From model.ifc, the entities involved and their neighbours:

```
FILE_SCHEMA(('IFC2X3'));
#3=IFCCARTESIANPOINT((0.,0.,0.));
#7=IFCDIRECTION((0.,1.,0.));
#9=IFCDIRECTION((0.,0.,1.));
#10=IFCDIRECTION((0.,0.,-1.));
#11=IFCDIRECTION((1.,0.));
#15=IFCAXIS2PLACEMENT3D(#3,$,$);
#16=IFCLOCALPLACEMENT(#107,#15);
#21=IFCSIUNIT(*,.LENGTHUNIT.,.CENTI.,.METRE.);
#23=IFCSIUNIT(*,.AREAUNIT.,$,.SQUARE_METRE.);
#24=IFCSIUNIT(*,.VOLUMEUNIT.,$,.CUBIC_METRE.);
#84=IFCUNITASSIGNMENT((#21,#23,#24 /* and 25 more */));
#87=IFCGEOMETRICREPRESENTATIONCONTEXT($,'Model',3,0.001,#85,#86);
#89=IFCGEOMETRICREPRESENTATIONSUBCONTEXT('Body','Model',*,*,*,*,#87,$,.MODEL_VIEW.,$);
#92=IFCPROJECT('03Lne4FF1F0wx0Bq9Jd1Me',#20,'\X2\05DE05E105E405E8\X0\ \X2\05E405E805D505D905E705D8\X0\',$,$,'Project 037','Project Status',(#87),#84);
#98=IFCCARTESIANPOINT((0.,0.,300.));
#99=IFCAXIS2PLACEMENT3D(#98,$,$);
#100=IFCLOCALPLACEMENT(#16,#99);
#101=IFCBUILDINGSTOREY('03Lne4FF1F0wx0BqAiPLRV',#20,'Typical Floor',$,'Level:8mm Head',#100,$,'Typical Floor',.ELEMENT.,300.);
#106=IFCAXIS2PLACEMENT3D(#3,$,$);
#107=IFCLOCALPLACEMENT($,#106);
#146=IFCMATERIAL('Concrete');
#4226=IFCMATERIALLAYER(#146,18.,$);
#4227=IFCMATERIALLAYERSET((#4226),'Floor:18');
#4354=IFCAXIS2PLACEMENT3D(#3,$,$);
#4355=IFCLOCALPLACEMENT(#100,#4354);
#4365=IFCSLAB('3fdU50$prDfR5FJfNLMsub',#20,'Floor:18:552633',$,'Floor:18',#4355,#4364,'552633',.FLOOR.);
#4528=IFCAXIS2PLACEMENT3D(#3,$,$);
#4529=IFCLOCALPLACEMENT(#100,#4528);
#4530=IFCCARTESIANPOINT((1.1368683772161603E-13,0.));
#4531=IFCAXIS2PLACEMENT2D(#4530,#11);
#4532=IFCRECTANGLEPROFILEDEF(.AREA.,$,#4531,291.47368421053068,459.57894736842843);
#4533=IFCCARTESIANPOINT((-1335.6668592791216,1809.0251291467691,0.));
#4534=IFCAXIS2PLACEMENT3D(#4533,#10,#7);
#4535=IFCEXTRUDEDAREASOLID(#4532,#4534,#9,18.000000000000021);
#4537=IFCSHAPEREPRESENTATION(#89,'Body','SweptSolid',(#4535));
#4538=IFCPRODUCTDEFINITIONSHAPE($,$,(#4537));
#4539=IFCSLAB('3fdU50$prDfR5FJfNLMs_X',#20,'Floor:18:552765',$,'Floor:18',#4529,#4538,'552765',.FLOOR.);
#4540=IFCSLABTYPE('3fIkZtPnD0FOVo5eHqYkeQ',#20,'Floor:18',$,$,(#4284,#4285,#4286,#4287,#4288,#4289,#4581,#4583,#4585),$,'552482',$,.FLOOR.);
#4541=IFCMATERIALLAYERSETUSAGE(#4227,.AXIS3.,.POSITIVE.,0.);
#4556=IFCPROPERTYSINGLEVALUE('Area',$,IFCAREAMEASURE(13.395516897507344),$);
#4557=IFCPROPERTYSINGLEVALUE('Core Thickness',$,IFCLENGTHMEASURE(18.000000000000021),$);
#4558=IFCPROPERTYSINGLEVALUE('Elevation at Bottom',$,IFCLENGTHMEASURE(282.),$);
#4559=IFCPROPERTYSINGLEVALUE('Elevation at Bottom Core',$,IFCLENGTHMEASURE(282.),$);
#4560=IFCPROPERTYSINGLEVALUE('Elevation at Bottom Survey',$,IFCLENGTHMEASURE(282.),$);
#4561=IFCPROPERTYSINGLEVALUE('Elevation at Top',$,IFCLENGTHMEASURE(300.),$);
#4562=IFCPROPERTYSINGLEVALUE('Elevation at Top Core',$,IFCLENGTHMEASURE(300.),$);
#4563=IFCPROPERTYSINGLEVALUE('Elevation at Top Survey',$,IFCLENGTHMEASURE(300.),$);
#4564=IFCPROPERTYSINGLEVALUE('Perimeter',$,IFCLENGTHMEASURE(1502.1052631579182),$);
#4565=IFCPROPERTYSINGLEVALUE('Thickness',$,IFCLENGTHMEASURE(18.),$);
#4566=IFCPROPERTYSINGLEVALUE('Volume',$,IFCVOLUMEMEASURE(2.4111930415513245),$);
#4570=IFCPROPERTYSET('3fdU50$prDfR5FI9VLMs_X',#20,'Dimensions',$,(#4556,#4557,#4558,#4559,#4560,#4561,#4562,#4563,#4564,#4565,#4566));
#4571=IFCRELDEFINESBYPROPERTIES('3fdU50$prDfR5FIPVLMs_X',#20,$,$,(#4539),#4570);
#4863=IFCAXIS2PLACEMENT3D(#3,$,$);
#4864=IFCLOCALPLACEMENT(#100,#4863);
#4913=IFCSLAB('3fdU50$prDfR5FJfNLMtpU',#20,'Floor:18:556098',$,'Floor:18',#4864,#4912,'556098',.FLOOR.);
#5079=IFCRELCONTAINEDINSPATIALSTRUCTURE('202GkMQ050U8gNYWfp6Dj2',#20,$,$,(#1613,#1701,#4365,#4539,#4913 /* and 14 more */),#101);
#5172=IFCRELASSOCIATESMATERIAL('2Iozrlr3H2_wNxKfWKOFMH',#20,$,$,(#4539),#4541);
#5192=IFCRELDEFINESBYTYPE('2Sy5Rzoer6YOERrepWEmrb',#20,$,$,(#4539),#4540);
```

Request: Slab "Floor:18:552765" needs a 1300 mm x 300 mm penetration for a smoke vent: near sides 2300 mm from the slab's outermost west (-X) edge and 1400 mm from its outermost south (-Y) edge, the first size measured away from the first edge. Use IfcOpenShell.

```python
import numpy as np
import ifcopenshell
import ifcopenshell.api.feature
import ifcopenshell.api.geometry
import ifcopenshell.api.pset
import ifcopenshell.api.root
import ifcopenshell.geom
import ifcopenshell.util.element
import ifcopenshell.util.placement
import ifcopenshell.util.representation
import ifcopenshell.util.shape
import ifcopenshell.util.unit

model = ifcopenshell.open("model.ifc")
unit_scale = ifcopenshell.util.unit.calculate_unit_scale(model)
area_scale = ifcopenshell.util.unit.calculate_unit_scale(model, "AREAUNIT")
volume_scale = ifcopenshell.util.unit.calculate_unit_scale(model, "VOLUMEUNIT")
settings = ifcopenshell.geom.settings()


def volume(element):
    """Net volume in cubic metres, openings subtracted."""
    shape = ifcopenshell.geom.create_shape(settings, element)
    return ifcopenshell.util.shape.get_volume(shape.geometry)


slab = model.by_guid("3fdU50$prDfR5FJfNLMs_X")
before = volume(slab)

# Extent in the slab's own axes, in metres. The edges named are its -X and -Y sides.
slab_shape = ifcopenshell.geom.create_shape(settings, slab)
vertices = ifcopenshell.util.shape.get_vertices(slab_shape.geometry)
x_min, y_min, bottom = vertices.min(axis=0)
top = vertices[:, 2].max()

opening = ifcopenshell.api.root.create_entity(model, ifc_class="IfcOpeningElement", name="Smoke vent opening")
context = ifcopenshell.util.representation.get_context(model, "Model", "Body", "MODEL_VIEW")
width, depth = 1.3, 0.3
outline = [(0.0, 0.0), (width, 0.0), (width, depth), (0.0, depth), (0.0, 0.0)]
# Overshoot both faces by 50 mm so the cut is clean.
shape = ifcopenshell.api.geometry.add_slab_representation(
    model, context=context, depth=top - bottom + 0.1, polyline=outline
)
ifcopenshell.api.geometry.assign_representation(model, product=opening, representation=shape)

matrix = ifcopenshell.util.placement.get_local_placement(slab.ObjectPlacement)
matrix[:, 3] = matrix @ np.append(np.array([x_min + 2.3, y_min + 1.4, bottom - 0.05]) / unit_scale, 1.0)
ifcopenshell.api.geometry.edit_object_placement(model, product=opening, matrix=matrix, is_si=False)
ifcopenshell.api.feature.add_feature(model, feature=opening, element=slab)

after = volume(slab)

# Update the slab's stored quantities.
pset = model.by_id(ifcopenshell.util.element.get_pset(slab, "Dimensions", should_inherit=False)["id"])
ifcopenshell.api.pset.edit_pset(model, pset=pset, properties={
    "Area": model.create_entity("IfcAreaMeasure", after / (top - bottom) / area_scale),
    "Volume": model.create_entity("IfcVolumeMeasure", after / volume_scale),
})

print(f"slab volume {before:.3f} -> {after:.3f} m3")

model.write("model_rev.ifc")
```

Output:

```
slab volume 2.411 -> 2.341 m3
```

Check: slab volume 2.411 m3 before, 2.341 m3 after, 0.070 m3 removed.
